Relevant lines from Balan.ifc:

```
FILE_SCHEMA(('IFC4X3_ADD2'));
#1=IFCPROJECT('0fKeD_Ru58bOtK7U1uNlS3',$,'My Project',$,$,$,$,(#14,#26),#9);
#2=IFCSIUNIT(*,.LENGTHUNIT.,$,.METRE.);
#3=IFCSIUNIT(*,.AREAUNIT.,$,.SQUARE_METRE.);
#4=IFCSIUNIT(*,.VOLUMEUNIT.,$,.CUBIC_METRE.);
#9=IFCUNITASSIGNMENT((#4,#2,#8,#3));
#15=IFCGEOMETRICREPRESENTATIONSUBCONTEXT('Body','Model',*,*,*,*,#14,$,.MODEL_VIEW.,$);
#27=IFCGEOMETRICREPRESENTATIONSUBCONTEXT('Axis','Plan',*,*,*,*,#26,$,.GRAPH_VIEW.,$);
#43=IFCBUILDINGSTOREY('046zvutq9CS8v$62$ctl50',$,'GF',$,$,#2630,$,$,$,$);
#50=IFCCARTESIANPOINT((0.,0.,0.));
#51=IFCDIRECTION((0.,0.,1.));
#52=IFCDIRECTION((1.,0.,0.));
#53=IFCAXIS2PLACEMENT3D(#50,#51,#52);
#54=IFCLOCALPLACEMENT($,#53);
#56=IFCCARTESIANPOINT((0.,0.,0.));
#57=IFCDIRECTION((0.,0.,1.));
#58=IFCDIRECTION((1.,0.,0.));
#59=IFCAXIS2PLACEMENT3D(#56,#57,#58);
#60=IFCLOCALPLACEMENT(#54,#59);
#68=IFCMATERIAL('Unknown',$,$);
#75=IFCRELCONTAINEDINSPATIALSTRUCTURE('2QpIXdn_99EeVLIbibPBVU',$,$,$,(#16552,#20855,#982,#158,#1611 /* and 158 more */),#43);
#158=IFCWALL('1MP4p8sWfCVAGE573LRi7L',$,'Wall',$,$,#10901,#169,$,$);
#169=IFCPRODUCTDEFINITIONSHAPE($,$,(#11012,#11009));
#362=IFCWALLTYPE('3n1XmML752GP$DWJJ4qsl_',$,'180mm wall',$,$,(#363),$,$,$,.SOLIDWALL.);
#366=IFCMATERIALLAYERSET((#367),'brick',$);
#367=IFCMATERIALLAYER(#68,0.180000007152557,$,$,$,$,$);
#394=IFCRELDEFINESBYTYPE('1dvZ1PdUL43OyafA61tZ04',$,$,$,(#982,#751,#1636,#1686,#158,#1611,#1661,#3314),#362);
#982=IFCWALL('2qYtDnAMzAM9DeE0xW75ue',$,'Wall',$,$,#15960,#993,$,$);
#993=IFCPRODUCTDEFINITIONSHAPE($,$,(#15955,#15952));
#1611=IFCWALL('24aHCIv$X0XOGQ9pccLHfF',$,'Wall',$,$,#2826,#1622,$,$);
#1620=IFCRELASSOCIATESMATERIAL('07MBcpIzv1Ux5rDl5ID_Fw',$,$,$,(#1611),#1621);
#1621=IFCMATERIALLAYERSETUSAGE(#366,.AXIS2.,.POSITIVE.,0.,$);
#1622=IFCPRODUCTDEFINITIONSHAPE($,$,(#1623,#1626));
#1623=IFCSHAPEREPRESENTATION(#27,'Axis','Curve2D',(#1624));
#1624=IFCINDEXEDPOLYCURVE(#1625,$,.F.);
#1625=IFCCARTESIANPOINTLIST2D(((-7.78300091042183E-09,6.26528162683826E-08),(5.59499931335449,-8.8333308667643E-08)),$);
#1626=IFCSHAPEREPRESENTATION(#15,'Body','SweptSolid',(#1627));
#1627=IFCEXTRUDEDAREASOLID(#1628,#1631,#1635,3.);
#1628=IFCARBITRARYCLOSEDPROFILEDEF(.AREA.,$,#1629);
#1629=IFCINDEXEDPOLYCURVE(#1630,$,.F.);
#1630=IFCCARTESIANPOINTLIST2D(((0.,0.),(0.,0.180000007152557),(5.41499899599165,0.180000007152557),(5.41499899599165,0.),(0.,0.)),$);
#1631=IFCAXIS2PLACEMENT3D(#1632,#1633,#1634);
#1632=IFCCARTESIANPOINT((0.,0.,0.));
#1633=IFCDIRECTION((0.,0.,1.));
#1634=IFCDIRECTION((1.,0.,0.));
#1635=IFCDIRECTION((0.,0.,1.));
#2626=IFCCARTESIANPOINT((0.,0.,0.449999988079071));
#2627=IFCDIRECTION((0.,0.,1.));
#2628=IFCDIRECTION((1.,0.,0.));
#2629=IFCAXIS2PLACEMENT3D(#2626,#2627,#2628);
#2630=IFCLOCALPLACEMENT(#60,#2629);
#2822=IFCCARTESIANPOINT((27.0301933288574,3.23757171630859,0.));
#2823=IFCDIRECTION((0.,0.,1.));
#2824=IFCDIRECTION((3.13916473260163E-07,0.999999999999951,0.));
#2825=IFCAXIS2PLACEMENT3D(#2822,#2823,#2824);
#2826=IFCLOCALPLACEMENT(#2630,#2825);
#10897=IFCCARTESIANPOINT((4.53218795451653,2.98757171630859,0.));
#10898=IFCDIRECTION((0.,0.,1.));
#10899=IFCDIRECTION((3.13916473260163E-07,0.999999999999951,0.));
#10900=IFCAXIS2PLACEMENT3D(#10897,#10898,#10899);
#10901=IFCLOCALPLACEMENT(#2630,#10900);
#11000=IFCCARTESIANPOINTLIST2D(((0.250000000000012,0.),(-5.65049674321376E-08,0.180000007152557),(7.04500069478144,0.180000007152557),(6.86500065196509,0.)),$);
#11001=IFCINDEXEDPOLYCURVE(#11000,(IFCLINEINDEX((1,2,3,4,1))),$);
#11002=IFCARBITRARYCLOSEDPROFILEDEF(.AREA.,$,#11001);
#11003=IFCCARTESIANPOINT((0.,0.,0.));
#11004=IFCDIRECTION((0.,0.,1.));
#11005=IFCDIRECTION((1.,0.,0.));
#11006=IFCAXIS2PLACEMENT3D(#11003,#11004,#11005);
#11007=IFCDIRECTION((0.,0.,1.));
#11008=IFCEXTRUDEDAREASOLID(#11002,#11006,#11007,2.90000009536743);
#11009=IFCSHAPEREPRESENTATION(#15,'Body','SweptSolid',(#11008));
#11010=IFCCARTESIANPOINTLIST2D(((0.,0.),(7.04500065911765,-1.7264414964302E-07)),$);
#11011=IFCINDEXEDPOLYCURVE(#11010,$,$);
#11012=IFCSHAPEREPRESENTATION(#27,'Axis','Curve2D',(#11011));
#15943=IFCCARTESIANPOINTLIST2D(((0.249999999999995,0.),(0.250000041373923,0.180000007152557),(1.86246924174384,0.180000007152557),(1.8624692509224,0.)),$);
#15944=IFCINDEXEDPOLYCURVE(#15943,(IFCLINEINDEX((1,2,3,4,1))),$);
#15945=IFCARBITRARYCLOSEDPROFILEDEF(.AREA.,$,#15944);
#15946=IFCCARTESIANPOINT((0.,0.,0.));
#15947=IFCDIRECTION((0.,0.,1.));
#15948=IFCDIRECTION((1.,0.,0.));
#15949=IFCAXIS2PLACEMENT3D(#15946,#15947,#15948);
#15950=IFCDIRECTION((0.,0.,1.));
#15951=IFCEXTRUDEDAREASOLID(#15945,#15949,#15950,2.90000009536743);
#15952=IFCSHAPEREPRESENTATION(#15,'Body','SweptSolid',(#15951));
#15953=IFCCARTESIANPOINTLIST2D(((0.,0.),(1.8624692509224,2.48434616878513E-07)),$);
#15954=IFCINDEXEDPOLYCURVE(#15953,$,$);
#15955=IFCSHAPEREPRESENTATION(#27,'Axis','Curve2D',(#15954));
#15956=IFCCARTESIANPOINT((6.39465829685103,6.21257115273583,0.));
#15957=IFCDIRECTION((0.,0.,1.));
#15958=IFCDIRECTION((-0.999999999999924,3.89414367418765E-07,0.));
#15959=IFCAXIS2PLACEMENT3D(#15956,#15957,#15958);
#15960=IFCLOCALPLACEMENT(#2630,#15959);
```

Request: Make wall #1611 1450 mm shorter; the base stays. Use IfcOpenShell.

```python
import ifcopenshell
import ifcopenshell.geom
import ifcopenshell.util.representation
import ifcopenshell.util.shape

model = ifcopenshell.open("Balan.ifc")
settings = ifcopenshell.geom.settings()


def volume(element):
    """Net volume in cubic metres, openings subtracted."""
    shape = ifcopenshell.geom.create_shape(settings, element)
    return ifcopenshell.util.shape.get_volume(shape.geometry)


wall = model.by_id(1611)
before = volume(wall)

body = ifcopenshell.util.representation.get_representation(wall, "Model", "Body")
solid = body.Items[0]
old_height = solid.Depth
solid.Depth -= 1.45
after = volume(wall)

print(f"height {old_height:g} -> {solid.Depth:g}, volume {before:.3f} -> {after:.3f} m3")

model.write("Balan_v2.ifc")
```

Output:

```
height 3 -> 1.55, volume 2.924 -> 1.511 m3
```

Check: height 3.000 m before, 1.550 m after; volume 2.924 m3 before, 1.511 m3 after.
